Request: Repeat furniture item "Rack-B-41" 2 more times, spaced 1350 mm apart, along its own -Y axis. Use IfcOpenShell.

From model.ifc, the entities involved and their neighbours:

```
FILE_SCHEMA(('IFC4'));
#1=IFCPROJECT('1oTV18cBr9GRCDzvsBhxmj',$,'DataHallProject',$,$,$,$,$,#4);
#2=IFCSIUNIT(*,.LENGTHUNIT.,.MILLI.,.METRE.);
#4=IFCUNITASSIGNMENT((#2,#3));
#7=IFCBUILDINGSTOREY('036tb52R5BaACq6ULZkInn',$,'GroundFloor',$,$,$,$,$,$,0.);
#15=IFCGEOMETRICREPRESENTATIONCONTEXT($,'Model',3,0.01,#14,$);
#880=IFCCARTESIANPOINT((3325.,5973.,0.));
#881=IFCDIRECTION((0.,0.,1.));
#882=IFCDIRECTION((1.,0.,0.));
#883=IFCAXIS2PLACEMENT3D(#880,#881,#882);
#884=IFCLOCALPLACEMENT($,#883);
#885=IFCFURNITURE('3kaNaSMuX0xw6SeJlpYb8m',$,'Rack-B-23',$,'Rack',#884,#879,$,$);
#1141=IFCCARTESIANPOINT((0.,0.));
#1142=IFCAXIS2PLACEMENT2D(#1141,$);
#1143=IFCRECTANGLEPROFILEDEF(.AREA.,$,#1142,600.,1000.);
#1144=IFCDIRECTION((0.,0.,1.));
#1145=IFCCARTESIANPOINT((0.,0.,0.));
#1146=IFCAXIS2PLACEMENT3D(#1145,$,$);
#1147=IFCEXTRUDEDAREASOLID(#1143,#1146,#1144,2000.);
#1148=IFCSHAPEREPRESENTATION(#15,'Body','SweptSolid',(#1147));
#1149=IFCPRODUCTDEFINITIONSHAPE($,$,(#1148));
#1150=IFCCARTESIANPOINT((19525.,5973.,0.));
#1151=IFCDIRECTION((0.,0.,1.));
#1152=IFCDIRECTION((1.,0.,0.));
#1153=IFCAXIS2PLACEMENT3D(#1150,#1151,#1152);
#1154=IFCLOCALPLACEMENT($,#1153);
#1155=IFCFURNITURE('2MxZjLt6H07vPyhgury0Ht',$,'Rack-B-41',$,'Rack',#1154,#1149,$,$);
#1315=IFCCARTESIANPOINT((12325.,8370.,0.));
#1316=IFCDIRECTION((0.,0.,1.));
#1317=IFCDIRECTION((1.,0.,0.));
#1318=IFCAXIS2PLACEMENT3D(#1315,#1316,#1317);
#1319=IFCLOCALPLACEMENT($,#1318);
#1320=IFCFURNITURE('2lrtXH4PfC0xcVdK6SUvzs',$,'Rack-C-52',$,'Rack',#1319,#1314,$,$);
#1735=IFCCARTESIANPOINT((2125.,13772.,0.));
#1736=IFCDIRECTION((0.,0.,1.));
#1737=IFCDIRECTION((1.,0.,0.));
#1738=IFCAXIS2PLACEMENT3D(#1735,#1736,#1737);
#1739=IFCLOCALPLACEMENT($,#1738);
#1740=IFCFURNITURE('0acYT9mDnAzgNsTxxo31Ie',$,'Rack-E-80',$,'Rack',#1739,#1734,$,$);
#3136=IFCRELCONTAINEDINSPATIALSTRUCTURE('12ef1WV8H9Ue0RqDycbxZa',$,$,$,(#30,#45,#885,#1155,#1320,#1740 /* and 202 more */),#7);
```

```python
import ifcopenshell
import ifcopenshell.api.geometry
import ifcopenshell.api.root
import ifcopenshell.util.element
import ifcopenshell.util.placement
import ifcopenshell.util.unit

model = ifcopenshell.open("model.ifc")
unit_scale = ifcopenshell.util.unit.calculate_unit_scale(model)

source = model.by_guid("2MxZjLt6H07vPyhgury0Ht")
base = ifcopenshell.util.placement.get_local_placement(source.ObjectPlacement)
step = -base[:3, 1] * 1.35 / unit_scale

for i in range(1, 3):
    copy = ifcopenshell.api.root.copy_class(model, product=source)
    copy.Representation = ifcopenshell.util.element.copy_deep(
        model, source.Representation, exclude=["IfcGeometricRepresentationContext", "IfcRepresentationMap"]
    )
    matrix = base.copy()
    matrix[:3, 3] += i * step
    print("added at", matrix[:3, 3].round(3) + 0.0)
    ifcopenshell.api.geometry.edit_object_placement(model, product=copy, matrix=matrix, is_si=False)

model.write("model_edited.ifc")
```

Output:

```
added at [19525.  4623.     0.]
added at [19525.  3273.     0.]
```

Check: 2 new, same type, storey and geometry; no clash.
